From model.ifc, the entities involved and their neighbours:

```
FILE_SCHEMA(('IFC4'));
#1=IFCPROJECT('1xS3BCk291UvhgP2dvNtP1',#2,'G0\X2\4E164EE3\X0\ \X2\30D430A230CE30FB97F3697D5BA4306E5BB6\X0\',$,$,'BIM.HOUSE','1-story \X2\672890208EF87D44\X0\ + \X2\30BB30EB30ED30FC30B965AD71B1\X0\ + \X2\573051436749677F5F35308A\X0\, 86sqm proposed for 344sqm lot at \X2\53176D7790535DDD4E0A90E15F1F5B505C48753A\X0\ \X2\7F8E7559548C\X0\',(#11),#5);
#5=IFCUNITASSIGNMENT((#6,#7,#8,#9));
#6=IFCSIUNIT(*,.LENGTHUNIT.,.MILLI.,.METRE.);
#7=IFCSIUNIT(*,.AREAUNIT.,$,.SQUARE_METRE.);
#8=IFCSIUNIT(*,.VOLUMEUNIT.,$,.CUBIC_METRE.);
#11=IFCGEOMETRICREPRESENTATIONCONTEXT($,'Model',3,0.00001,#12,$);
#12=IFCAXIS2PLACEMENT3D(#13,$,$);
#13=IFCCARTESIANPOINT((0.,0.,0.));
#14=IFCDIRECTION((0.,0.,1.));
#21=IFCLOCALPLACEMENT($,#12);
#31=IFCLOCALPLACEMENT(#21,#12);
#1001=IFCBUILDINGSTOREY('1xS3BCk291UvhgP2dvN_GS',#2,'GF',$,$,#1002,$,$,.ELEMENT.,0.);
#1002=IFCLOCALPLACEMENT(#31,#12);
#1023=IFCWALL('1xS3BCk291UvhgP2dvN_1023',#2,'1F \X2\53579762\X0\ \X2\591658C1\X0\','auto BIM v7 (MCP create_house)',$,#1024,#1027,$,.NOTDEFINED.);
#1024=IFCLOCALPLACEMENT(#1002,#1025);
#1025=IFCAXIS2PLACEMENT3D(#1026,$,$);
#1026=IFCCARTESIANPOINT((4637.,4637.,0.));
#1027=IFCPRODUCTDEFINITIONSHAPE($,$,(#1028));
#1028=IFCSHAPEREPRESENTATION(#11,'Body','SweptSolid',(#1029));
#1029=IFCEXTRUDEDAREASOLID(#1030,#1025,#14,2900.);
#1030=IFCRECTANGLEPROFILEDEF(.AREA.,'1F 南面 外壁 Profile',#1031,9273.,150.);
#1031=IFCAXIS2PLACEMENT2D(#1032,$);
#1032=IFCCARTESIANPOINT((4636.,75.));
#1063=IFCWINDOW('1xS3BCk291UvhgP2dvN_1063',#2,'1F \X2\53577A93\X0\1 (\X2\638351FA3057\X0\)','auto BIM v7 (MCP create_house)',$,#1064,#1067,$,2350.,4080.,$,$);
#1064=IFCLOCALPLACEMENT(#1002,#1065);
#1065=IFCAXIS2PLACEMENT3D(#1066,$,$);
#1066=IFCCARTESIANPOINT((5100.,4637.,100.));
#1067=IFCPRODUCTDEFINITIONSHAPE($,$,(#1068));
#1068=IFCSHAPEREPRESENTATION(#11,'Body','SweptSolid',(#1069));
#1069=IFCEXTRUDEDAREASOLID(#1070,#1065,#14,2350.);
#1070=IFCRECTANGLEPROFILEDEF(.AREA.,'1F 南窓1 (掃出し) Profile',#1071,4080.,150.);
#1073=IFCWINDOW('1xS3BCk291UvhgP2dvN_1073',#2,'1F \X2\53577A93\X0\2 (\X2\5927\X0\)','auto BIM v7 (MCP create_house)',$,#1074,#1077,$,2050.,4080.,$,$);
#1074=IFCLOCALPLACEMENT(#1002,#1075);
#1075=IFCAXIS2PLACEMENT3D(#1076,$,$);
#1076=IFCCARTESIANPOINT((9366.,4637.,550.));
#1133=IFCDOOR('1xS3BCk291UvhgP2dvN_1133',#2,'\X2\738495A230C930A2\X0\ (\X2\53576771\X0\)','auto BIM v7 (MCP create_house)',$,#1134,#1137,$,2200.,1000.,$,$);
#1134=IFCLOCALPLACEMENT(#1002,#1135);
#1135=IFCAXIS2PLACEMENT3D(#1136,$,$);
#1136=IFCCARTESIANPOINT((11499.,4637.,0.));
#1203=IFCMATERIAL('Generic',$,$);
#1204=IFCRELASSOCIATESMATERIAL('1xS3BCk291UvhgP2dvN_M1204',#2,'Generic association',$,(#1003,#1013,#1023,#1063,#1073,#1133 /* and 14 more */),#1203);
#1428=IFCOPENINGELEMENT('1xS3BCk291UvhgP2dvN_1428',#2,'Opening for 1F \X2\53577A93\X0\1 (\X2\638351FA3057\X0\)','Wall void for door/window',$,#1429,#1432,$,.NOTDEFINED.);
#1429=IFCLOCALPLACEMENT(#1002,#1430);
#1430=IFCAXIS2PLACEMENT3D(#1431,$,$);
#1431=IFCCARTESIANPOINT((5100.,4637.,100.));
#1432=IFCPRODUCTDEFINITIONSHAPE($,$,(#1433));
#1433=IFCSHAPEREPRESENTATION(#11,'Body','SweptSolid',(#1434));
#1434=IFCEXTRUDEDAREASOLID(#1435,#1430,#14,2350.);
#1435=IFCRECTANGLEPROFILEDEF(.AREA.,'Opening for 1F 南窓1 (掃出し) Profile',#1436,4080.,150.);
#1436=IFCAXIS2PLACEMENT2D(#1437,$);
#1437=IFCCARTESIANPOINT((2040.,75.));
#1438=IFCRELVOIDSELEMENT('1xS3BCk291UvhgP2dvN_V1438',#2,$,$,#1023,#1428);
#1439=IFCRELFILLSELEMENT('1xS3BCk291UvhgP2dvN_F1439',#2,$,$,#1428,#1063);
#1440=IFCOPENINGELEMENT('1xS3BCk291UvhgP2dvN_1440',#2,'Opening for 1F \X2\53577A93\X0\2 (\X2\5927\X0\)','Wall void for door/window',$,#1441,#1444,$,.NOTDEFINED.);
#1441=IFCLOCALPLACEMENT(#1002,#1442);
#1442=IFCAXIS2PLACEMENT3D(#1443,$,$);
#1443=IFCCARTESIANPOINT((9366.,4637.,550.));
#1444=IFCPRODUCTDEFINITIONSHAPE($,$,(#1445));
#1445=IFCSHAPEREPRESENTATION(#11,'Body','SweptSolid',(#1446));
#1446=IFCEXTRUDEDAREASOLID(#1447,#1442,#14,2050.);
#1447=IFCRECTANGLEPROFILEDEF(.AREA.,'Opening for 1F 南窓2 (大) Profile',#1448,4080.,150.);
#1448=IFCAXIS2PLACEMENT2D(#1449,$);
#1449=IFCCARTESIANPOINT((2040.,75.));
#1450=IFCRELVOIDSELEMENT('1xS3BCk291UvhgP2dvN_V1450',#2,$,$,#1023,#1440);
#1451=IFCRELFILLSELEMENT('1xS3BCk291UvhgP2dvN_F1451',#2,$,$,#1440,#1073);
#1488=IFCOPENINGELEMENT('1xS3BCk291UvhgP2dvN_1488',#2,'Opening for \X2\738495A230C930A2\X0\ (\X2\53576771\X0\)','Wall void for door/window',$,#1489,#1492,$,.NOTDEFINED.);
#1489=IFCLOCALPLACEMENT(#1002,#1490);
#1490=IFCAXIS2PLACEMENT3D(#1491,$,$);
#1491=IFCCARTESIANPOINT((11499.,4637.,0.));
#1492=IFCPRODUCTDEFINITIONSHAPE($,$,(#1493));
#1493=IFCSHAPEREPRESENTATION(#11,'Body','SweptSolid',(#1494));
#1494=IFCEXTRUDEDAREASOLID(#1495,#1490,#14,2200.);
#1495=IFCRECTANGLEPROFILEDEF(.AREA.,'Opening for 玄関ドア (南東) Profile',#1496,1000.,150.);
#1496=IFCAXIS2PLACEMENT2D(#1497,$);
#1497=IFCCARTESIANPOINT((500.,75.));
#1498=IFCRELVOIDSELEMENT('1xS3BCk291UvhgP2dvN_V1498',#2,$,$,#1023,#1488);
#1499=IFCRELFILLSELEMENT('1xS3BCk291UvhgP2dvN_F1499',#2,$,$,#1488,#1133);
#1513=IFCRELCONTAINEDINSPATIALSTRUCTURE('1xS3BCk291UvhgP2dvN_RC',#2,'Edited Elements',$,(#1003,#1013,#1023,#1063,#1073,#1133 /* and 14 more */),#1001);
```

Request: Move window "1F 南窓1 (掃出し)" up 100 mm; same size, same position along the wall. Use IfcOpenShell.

```python
import numpy as np
import ifcopenshell
import ifcopenshell.api.geometry
import ifcopenshell.util.placement
import ifcopenshell.util.unit

model = ifcopenshell.open("model.ifc")
unit_scale = ifcopenshell.util.unit.calculate_unit_scale(model)

window = model.by_id(1063)
opening = window.FillsVoids[0].RelatingOpeningElement
dz = 0.1 / unit_scale

shift = np.array([0.0, 0.0, dz])
# The window is not placed relative to its opening, so move both.
for product in (opening, window):
    matrix = ifcopenshell.util.placement.get_local_placement(product.ObjectPlacement)
    matrix[:3, 3] += shift
    ifcopenshell.api.geometry.edit_object_placement(model, product=product, matrix=matrix, is_si=False)

print(f"moved by {dz * unit_scale:+.3f} m")

model.write("model_edited.ifc")
```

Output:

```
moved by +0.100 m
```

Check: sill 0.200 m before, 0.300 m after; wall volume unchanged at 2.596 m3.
